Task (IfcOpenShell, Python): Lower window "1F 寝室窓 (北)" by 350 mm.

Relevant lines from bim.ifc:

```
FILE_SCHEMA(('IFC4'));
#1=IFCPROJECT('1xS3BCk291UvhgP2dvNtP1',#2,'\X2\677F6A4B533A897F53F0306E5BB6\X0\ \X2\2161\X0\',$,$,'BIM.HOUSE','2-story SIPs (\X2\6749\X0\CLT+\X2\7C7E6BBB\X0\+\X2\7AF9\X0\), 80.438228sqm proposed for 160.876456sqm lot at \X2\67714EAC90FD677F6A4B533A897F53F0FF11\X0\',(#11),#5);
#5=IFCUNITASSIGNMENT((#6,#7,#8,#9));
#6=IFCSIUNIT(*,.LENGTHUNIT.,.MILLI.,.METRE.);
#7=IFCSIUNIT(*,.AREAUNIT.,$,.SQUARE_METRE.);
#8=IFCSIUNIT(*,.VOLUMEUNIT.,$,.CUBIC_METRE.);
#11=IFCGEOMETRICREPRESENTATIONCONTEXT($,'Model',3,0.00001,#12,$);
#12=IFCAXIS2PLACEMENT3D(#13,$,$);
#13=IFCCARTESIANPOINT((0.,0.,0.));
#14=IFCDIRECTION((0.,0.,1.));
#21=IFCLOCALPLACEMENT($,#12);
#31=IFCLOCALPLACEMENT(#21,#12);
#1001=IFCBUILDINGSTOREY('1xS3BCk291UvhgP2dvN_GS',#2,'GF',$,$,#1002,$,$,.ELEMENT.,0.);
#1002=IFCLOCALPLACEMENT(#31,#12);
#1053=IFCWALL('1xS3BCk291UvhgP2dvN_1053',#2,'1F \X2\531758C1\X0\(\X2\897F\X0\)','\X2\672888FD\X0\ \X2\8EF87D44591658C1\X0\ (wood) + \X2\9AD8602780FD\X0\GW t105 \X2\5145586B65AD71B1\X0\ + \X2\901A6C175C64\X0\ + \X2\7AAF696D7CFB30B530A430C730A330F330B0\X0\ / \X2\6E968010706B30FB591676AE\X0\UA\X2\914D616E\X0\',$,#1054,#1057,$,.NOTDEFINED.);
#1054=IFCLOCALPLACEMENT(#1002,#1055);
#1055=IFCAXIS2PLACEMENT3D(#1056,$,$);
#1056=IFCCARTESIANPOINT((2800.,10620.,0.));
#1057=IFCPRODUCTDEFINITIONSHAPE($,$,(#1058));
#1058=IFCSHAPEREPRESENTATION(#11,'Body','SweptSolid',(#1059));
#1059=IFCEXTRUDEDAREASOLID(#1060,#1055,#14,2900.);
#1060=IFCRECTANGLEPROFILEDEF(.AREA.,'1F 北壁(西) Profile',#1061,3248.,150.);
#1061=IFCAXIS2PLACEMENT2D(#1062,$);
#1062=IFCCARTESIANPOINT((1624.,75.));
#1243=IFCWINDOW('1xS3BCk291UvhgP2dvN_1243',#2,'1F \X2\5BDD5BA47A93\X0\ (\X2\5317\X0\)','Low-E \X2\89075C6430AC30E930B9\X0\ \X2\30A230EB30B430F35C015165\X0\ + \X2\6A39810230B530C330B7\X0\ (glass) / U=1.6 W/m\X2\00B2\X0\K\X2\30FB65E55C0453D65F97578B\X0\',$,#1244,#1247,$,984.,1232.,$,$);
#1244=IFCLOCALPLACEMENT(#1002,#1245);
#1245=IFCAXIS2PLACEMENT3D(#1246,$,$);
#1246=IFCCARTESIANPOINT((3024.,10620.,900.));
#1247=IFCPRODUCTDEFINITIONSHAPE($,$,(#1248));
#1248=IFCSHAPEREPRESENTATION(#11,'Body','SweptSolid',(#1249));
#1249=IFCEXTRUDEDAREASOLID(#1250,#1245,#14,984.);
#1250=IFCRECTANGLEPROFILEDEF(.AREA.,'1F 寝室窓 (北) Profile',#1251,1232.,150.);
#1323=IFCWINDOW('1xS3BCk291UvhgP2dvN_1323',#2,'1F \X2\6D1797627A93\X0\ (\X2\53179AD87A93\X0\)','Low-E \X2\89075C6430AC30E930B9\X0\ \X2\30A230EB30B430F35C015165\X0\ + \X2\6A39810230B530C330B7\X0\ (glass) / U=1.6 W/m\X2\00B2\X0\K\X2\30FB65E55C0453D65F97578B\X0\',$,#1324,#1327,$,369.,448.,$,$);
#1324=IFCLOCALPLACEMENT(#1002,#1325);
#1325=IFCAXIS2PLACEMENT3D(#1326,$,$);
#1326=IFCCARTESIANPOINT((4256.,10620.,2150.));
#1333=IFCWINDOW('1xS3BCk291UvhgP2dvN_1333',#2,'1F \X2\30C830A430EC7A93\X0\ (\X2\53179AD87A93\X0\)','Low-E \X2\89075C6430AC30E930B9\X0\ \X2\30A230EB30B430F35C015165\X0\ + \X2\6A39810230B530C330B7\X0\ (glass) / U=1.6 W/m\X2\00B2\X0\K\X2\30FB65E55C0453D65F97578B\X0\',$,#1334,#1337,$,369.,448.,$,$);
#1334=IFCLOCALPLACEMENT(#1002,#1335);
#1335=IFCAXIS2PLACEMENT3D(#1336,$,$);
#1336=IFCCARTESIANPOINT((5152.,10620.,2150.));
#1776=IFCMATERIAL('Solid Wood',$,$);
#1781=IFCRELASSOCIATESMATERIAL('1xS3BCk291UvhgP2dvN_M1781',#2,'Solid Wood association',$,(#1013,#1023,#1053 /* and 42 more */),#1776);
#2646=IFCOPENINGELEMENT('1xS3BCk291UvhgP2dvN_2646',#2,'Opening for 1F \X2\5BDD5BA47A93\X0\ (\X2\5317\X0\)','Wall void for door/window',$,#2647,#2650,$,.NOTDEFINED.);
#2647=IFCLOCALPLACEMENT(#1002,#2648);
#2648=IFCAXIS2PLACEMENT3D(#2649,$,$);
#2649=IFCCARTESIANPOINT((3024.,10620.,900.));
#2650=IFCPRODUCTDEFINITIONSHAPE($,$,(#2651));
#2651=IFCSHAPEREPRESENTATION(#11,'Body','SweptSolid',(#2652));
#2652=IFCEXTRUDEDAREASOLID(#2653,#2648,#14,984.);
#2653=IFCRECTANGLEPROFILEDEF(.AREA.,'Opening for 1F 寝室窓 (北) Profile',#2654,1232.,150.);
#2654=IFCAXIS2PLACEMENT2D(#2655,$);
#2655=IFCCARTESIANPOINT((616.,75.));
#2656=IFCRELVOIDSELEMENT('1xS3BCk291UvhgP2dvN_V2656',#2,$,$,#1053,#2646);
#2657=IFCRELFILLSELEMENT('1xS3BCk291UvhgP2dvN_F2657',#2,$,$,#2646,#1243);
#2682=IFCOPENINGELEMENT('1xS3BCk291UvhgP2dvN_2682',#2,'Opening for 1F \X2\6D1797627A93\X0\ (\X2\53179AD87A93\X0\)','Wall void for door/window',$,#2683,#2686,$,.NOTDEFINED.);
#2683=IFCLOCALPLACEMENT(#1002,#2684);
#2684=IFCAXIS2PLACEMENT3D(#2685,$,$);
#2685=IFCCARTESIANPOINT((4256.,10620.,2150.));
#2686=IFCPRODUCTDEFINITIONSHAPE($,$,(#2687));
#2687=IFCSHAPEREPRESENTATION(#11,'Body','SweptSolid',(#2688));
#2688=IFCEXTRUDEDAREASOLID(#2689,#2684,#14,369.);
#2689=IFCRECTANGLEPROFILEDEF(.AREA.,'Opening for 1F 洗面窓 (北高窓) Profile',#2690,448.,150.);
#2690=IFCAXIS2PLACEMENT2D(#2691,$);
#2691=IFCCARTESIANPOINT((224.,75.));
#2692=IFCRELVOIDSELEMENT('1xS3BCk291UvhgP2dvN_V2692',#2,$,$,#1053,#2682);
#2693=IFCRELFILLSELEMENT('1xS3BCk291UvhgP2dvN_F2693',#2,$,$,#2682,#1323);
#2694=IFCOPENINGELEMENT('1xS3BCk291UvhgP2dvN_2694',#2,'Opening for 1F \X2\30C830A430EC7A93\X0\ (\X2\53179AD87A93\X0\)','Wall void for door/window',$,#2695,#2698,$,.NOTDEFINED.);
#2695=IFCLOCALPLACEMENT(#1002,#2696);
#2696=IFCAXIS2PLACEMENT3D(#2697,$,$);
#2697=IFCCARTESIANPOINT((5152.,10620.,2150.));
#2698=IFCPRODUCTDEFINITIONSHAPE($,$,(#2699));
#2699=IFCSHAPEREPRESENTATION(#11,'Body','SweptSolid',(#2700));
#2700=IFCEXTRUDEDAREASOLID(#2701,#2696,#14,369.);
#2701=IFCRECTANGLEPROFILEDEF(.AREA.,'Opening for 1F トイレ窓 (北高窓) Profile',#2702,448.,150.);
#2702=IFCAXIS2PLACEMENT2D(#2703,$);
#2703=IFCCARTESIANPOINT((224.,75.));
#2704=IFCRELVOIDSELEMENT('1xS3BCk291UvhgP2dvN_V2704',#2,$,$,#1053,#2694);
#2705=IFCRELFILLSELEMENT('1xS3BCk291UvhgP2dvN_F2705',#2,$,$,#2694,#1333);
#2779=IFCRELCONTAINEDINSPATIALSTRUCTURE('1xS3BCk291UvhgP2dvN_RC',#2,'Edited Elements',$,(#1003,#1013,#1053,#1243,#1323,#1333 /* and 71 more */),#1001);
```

```python
import numpy as np
import ifcopenshell
import ifcopenshell.api.geometry
import ifcopenshell.util.placement
import ifcopenshell.util.unit

model = ifcopenshell.open("bim.ifc")
unit_scale = ifcopenshell.util.unit.calculate_unit_scale(model)

window = model.by_guid("1xS3BCk291UvhgP2dvN_1243")
opening = window.FillsVoids[0].RelatingOpeningElement
dz = -0.35 / unit_scale

shift = np.array([0.0, 0.0, dz])
# The window is not placed relative to its opening, so move both.
for product in (opening, window):
    matrix = ifcopenshell.util.placement.get_local_placement(product.ObjectPlacement)
    matrix[:3, 3] += shift
    ifcopenshell.api.geometry.edit_object_placement(model, product=product, matrix=matrix, is_si=False)

print(f"moved by {dz * unit_scale:+.3f} m")

model.write("bim-out.ifc")
```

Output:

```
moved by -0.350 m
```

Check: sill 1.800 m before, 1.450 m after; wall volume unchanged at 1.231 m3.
